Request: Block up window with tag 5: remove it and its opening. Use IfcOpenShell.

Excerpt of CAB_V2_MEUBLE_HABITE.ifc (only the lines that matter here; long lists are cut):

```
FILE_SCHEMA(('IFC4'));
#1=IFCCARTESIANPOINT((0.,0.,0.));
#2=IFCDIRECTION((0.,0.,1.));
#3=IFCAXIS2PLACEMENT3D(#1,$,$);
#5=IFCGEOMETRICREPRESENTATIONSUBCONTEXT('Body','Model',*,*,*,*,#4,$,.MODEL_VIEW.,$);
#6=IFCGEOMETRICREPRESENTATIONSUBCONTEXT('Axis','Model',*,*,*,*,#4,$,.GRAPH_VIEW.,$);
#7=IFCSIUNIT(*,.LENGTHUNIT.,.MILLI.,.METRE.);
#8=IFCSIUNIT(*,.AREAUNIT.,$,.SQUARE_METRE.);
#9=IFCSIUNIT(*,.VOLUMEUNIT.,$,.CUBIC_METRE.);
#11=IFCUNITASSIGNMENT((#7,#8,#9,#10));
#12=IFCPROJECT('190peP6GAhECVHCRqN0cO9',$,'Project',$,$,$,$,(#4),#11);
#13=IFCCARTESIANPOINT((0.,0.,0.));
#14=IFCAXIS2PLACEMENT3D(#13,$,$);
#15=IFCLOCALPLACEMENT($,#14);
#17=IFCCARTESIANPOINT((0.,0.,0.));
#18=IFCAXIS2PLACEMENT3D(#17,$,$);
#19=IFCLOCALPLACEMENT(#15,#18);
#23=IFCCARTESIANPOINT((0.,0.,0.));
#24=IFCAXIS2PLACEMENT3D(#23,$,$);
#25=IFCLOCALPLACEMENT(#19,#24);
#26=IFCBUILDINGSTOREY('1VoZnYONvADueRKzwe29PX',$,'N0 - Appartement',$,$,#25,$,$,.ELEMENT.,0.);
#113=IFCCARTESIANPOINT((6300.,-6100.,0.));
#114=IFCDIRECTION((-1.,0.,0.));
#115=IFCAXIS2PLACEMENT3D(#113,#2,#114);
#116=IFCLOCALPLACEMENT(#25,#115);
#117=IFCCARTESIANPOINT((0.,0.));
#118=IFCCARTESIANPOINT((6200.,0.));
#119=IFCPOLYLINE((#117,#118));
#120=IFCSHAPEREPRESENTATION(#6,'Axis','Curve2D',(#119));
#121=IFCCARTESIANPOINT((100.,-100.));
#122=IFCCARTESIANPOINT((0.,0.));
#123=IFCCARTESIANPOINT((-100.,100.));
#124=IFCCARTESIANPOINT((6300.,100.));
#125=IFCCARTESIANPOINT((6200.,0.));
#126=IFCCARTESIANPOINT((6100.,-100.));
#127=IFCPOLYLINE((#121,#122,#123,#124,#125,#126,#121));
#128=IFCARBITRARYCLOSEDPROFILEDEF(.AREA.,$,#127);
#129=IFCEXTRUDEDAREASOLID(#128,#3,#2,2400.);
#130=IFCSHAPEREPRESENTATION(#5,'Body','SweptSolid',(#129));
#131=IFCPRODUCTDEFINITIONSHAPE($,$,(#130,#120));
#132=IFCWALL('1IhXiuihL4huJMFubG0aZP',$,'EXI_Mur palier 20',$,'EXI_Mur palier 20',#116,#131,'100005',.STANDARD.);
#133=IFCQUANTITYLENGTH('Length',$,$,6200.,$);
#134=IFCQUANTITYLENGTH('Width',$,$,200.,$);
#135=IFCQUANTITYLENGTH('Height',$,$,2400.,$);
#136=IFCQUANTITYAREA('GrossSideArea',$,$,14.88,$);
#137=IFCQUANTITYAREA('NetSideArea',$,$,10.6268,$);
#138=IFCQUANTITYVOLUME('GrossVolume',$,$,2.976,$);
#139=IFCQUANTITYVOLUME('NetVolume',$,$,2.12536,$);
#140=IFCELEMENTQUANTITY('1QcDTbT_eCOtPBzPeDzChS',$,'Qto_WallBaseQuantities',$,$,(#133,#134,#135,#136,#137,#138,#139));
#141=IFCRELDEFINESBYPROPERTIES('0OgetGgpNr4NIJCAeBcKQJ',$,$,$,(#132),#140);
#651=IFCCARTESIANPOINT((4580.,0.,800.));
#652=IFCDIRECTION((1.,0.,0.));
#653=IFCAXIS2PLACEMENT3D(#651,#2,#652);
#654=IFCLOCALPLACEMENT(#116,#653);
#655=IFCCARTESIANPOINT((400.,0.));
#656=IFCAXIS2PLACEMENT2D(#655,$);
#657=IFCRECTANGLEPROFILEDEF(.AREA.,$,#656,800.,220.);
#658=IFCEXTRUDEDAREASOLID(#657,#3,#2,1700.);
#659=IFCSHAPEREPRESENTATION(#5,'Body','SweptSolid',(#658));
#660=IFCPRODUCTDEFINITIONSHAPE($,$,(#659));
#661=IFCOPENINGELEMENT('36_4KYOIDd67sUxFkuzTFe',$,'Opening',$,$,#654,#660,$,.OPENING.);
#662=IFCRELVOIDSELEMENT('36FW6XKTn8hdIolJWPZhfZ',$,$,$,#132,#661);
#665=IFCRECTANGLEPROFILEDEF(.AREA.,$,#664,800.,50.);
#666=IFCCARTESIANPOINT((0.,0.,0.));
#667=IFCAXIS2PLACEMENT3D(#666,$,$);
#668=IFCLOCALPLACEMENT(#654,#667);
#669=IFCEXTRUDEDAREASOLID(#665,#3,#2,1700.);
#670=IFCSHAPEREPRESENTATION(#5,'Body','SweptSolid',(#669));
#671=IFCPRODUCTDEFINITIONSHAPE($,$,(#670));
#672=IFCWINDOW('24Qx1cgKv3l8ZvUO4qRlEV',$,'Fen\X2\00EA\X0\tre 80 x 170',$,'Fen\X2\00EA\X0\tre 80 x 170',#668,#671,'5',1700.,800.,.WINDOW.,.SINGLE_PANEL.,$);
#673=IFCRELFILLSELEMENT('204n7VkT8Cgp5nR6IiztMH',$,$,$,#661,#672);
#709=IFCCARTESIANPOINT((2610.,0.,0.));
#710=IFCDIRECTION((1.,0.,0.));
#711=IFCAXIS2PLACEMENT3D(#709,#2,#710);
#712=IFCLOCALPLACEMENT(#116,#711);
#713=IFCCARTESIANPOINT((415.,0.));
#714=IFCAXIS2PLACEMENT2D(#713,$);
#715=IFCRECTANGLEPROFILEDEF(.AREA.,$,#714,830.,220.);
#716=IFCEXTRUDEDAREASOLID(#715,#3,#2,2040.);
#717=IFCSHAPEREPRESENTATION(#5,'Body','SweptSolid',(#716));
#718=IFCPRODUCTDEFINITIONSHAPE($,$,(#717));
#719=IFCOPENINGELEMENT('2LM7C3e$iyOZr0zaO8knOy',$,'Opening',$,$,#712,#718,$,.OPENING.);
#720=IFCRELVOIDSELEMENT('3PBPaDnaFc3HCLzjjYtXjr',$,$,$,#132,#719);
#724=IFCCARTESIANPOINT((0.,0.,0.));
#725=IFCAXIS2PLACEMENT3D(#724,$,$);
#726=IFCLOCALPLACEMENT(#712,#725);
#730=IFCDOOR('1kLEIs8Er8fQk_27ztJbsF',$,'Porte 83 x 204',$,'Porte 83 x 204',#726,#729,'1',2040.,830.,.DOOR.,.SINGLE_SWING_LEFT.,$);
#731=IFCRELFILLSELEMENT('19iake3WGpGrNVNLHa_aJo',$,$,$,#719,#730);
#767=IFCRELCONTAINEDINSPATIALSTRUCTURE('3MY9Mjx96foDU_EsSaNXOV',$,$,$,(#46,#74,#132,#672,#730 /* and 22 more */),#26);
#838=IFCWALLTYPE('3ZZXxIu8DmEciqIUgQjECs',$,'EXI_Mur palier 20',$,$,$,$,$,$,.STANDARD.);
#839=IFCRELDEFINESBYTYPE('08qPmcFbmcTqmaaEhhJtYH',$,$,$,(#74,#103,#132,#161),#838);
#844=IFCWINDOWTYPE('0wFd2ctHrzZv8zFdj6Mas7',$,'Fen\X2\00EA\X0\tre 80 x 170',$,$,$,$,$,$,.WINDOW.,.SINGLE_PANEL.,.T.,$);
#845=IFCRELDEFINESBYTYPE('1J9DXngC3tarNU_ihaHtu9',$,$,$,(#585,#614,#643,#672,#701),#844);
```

```python
import ifcopenshell
import ifcopenshell.api.feature
import ifcopenshell.api.pset
import ifcopenshell.api.root
import ifcopenshell.geom
import ifcopenshell.util.element
import ifcopenshell.util.shape
import ifcopenshell.util.unit

model = ifcopenshell.open("CAB_V2_MEUBLE_HABITE.ifc")
area_scale = ifcopenshell.util.unit.calculate_unit_scale(model, "AREAUNIT")
volume_scale = ifcopenshell.util.unit.calculate_unit_scale(model, "VOLUMEUNIT")
settings = ifcopenshell.geom.settings()


def volume(element):
    """Net volume in cubic metres, openings subtracted."""
    shape = ifcopenshell.geom.create_shape(settings, element)
    return ifcopenshell.util.shape.get_volume(shape.geometry)


window = model.by_guid("24Qx1cgKv3l8ZvUO4qRlEV")
opening = window.FillsVoids[0].RelatingOpeningElement
wall = opening.VoidsElements[0].RelatingBuildingElement
before = volume(wall)

ifcopenshell.api.root.remove_product(model, product=window)
ifcopenshell.api.feature.remove_feature(model, feature=opening)

after = volume(wall)
thickness = 0.2  # wall thickness in metres

# Update the wall's stored quantities.
qto = model.by_id(ifcopenshell.util.element.get_pset(wall, "Qto_WallBaseQuantities", should_inherit=False)["id"])
ifcopenshell.api.pset.edit_qto(model, qto=qto, properties={
    "NetSideArea": after / thickness / area_scale,
    "NetVolume": after / volume_scale,
})

print(f"wall volume {before:.3f} -> {after:.3f} m3")

model.write("CAB_V2_MEUBLE_HABITE_updated.ifc")
```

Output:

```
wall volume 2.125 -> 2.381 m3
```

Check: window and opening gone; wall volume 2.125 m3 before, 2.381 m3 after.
